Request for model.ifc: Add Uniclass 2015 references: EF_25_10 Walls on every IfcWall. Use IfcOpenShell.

First a look at what the model holds.

```python
import ifcopenshell

model = ifcopenshell.open("model.ifc")
print(model.schema)
print("classifications:", [c.Name for c in model.by_type("IfcClassification")])
for ifc_class in ("IfcDoor", "IfcRoof", "IfcStair", "IfcWall", "IfcWindow"):
    print(ifc_class, len(model.by_type(ifc_class)))
```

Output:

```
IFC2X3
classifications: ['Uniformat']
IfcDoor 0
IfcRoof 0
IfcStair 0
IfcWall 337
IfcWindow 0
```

```python
import ifcopenshell
import ifcopenshell.api.classification

model = ifcopenshell.open("model.ifc")

# IFC2X3 requires Source and Edition and has no link from the project to the system.
system = model.create_entity("IfcClassification", Source="NBS", Edition="2015", Name="Uniclass 2015")

codes = {
    "IfcWall": ("EF_25_10", "Walls"),
}
for ifc_class, (code, name) in codes.items():
    products = model.by_type(ifc_class)
    ifcopenshell.api.classification.add_reference(
        model, products=products, classification=system, identification=code, name=name
    )
    print(code, len(products))

model.write("model_v2.ifc")
```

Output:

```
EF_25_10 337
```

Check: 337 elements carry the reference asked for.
